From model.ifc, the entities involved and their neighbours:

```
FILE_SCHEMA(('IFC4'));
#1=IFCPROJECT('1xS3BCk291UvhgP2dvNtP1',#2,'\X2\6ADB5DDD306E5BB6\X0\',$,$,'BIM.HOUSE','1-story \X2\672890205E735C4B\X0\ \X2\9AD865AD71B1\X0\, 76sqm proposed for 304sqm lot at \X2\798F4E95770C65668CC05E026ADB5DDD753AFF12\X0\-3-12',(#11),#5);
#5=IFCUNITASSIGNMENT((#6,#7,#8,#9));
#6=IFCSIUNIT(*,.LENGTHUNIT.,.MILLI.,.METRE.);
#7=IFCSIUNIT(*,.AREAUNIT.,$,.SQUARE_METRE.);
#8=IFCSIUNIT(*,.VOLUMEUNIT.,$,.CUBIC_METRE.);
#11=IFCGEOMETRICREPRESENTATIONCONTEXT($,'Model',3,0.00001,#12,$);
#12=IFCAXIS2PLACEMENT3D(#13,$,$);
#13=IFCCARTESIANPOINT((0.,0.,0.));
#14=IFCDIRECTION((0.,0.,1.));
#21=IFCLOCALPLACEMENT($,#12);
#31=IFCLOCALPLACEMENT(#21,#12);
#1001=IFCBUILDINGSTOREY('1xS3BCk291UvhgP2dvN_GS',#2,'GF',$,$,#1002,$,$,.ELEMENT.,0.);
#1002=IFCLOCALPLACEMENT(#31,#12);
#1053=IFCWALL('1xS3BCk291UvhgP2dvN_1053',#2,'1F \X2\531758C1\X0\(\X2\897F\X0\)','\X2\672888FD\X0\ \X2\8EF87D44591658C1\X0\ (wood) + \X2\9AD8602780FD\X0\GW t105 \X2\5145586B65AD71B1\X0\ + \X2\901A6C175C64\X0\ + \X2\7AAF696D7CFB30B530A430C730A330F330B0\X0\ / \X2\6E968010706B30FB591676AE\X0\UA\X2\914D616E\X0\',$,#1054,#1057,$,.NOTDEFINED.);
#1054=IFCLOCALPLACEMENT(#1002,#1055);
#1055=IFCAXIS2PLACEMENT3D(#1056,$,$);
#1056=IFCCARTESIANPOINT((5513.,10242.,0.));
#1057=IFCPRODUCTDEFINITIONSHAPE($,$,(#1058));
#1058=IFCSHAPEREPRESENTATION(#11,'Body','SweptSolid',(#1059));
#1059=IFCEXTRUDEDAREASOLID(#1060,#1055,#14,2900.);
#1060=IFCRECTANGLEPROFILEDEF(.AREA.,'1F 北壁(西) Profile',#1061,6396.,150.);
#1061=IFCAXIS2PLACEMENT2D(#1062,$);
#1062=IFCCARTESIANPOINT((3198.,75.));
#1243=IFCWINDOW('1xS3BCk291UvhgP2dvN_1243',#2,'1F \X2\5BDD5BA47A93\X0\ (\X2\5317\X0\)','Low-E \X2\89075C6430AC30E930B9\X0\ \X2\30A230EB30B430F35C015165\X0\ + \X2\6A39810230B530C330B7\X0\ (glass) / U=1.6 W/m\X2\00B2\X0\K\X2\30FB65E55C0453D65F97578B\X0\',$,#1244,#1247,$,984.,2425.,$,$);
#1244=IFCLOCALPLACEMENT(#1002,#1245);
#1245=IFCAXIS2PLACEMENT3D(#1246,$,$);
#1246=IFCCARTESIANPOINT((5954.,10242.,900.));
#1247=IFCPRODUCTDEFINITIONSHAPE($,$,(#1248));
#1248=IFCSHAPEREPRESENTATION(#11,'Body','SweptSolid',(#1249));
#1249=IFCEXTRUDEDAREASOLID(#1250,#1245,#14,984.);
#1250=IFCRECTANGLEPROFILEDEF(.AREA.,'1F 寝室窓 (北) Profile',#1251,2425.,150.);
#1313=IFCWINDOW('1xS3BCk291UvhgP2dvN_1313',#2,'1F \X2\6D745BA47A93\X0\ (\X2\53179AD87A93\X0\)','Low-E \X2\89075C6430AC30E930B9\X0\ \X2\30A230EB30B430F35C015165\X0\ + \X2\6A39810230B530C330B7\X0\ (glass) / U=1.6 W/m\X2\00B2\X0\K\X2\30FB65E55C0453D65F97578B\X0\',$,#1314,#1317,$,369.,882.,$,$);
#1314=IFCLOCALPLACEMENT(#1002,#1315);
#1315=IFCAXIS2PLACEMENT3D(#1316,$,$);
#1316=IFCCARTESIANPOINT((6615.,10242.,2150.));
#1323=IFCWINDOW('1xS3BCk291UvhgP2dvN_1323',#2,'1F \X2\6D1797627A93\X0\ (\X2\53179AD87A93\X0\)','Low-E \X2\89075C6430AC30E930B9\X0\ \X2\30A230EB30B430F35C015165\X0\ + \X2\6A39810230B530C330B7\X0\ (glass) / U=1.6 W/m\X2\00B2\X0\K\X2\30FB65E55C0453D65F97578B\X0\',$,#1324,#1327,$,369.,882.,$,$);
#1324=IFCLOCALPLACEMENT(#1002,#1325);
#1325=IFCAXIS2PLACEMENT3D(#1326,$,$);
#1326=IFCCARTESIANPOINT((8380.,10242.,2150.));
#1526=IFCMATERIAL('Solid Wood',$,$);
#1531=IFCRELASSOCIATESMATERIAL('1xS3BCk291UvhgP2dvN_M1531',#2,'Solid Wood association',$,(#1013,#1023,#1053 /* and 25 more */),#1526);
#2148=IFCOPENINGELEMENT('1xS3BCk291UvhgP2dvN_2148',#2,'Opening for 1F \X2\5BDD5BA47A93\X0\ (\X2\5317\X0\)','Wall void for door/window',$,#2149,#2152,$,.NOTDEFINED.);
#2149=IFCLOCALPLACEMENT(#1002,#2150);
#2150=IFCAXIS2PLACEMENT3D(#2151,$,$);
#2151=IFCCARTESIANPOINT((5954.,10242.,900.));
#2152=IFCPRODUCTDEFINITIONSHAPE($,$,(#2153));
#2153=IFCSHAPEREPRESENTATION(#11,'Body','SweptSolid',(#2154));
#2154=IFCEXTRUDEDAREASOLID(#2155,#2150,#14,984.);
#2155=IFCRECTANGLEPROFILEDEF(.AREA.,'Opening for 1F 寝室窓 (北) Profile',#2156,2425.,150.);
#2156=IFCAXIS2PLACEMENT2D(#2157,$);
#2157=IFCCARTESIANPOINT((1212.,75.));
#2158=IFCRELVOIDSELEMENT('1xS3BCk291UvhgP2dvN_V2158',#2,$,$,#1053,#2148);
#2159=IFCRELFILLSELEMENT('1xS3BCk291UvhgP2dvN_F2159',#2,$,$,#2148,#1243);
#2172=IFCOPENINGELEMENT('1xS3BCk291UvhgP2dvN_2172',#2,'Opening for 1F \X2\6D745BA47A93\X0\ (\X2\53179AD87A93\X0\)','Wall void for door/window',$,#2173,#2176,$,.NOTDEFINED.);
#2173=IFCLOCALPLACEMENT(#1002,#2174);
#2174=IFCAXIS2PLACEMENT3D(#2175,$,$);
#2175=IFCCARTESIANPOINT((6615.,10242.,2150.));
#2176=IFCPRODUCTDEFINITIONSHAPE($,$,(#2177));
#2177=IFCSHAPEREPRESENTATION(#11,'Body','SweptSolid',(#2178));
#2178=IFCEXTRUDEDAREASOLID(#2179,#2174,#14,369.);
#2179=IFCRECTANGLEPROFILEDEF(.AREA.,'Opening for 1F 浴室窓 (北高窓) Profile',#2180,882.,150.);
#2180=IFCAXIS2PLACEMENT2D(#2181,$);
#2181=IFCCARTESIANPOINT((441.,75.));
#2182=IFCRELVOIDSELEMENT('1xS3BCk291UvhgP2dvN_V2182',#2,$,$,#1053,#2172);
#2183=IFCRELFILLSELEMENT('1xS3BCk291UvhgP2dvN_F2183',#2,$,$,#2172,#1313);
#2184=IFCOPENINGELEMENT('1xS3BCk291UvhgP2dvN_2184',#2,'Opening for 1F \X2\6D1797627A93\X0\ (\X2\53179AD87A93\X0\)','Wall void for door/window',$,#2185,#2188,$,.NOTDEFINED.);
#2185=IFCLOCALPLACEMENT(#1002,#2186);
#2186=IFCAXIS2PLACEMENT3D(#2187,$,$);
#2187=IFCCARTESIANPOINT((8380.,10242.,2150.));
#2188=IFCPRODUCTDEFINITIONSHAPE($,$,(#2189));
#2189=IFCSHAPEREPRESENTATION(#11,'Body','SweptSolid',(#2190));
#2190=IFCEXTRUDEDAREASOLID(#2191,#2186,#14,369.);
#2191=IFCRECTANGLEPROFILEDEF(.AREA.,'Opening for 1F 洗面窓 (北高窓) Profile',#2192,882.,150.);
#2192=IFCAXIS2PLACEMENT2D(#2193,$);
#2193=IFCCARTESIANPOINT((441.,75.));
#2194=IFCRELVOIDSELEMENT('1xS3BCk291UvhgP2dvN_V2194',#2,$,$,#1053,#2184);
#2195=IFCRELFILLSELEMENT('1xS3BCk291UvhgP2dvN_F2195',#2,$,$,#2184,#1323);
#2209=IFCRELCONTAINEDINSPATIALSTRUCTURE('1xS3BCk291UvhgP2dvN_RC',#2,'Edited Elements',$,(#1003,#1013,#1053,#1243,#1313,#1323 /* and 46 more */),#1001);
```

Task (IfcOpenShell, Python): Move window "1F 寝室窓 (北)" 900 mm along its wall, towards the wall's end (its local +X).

```python
import ifcopenshell
import ifcopenshell.api.geometry
import ifcopenshell.util.placement
import ifcopenshell.util.unit

model = ifcopenshell.open("model.ifc")
unit_scale = ifcopenshell.util.unit.calculate_unit_scale(model)

window = model.by_id(1243)
opening = window.FillsVoids[0].RelatingOpeningElement
wall = opening.VoidsElements[0].RelatingBuildingElement

wall_matrix = ifcopenshell.util.placement.get_local_placement(wall.ObjectPlacement)
shift = wall_matrix[:3, 0] * 0.9 / unit_scale
before = ifcopenshell.util.placement.get_local_placement(window.ObjectPlacement)[:3, 3].copy()

# The window is not placed relative to its opening, so move both.
for product in (opening, window):
    matrix = ifcopenshell.util.placement.get_local_placement(product.ObjectPlacement)
    matrix[:3, 3] += shift
    ifcopenshell.api.geometry.edit_object_placement(model, product=product, matrix=matrix, is_si=False)

after = ifcopenshell.util.placement.get_local_placement(window.ObjectPlacement)[:3, 3]
print("window moved by", (after - before).round(3) + 0.0)

model.write("model-out.ifc")
```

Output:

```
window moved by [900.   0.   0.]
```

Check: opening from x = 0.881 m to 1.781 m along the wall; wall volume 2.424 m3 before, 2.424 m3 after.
